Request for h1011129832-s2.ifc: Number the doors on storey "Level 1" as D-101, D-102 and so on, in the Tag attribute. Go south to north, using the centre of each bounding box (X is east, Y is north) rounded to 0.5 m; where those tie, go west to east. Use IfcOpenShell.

First a look at what the model holds.

```python
import ifcopenshell
import ifcopenshell.util.element
import ifcopenshell.util.placement

model = ifcopenshell.open("h1011129832-s2.ifc")
print(model.schema)
storey = next(s for s in model.by_type("IfcBuildingStorey") if s.Name == "Level 1")
doors = [e for e in ifcopenshell.util.element.get_decomposition(storey) if e.is_a("IfcDoor")]
for e in sorted(doors, key=lambda e: e.id()):
    origin = ifcopenshell.util.placement.get_local_placement(e.ObjectPlacement)[:3, 3]
    print(e.id(), e.Tag, e.Name, origin.round(2) + 0.0, sep=" | ")
```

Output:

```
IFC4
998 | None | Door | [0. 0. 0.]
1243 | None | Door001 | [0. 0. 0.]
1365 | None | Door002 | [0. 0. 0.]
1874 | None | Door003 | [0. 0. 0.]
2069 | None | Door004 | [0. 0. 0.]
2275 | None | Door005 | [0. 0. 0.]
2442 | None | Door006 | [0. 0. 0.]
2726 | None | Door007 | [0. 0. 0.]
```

```python
import ifcopenshell
import ifcopenshell.geom
import ifcopenshell.util.element
import ifcopenshell.util.shape

model = ifcopenshell.open("h1011129832-s2.ifc")
settings = ifcopenshell.geom.settings()
settings.set("use-world-coords", True)


def centre(element):
    shape = ifcopenshell.geom.create_shape(settings, element)
    return ifcopenshell.util.shape.get_bbox_centroid(shape.geometry)


storey = next(s for s in model.by_type("IfcBuildingStorey") if s.Name == "Level 1")
doors = [e for e in ifcopenshell.util.element.get_decomposition(storey) if e.is_a("IfcDoor")]

# Insertion points can sit at a corner or the storey origin, so sort by the geometry (in metres).
centres = {e: centre(e) for e in doors}
doors.sort(key=lambda e: (round(centres[e][1] / 0.5), centres[e][0]))

for i, e in enumerate(doors, start=1):
    number = f"D-1{i:02d}"
    e.Tag = number
    print(e.id(), number)

model.write("h1011129832-s2-out.ifc")
```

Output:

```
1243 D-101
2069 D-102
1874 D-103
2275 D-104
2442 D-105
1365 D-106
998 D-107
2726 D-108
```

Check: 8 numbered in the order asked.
